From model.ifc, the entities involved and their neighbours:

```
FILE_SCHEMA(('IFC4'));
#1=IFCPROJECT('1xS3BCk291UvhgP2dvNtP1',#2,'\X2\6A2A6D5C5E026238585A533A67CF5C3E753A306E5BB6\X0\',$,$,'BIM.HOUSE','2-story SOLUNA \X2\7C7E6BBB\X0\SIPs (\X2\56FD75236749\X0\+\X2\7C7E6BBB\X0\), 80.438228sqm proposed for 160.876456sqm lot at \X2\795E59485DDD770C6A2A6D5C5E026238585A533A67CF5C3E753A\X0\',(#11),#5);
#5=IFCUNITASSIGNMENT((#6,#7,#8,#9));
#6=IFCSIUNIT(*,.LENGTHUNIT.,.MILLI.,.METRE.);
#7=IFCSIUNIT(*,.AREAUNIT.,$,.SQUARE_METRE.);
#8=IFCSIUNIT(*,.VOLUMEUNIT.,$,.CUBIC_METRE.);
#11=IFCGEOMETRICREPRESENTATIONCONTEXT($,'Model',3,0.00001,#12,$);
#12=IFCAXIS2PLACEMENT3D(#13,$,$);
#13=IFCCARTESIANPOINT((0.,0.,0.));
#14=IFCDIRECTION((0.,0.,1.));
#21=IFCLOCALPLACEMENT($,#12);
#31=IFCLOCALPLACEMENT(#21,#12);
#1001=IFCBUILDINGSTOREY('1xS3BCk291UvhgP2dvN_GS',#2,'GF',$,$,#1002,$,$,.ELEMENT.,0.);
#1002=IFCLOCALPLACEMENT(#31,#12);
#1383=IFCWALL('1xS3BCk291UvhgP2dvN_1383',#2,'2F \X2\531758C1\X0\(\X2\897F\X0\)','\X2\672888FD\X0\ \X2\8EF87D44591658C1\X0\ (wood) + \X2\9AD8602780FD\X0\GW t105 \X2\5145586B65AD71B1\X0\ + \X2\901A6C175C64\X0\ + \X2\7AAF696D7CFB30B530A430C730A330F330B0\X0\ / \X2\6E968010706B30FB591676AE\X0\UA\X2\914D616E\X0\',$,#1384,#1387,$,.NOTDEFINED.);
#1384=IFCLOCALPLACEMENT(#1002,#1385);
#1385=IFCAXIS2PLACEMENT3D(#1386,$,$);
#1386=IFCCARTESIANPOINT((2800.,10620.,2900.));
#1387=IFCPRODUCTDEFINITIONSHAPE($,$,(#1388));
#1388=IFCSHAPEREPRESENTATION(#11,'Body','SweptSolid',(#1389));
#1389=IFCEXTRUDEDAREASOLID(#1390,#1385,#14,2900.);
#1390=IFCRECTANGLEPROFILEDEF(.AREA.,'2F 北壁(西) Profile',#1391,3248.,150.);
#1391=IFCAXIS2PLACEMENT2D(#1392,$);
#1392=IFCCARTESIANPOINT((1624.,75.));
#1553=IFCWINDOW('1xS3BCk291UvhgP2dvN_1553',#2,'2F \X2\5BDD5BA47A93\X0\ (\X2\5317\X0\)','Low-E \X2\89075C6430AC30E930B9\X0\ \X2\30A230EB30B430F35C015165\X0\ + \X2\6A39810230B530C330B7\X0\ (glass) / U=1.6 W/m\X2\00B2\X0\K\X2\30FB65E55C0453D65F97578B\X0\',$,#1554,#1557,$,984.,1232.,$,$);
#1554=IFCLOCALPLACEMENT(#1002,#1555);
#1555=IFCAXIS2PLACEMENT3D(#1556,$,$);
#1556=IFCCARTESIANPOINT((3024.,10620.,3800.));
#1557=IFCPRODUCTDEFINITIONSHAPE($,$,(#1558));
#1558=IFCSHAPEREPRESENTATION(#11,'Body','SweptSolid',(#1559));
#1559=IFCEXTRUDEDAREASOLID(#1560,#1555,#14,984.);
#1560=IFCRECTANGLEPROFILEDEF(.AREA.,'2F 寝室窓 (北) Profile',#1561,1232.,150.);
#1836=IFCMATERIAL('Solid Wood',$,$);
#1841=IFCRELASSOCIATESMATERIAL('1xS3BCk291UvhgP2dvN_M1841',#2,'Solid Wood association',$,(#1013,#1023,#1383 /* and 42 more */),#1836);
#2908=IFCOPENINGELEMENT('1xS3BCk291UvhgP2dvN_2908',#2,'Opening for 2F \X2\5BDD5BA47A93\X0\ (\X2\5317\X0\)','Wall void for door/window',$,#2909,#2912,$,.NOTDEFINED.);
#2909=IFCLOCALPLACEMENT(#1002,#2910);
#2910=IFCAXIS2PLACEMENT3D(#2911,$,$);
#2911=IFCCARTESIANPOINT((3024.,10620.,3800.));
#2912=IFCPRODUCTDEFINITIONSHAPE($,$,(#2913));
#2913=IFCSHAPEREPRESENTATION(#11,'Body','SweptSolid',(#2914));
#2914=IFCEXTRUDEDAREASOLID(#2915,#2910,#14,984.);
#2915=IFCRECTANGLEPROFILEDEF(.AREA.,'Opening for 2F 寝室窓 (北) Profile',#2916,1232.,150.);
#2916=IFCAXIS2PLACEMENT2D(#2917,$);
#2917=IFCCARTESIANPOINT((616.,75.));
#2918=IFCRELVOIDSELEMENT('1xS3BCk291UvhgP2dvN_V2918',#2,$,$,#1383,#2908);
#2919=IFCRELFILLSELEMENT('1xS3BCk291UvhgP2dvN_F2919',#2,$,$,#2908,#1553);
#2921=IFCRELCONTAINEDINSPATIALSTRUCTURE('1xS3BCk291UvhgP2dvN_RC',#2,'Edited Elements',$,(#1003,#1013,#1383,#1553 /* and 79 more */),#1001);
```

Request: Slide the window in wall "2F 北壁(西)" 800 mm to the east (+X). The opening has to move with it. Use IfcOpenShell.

```python
import ifcopenshell
import ifcopenshell.api.geometry
import ifcopenshell.util.placement

model = ifcopenshell.open("model.ifc")

window = model.by_guid("1xS3BCk291UvhgP2dvN_1553")
opening = window.FillsVoids[0].RelatingOpeningElement
wall = opening.VoidsElements[0].RelatingBuildingElement

wall_matrix = ifcopenshell.util.placement.get_local_placement(wall.ObjectPlacement)
shift = wall_matrix[:3, 0] * 800.0
before = ifcopenshell.util.placement.get_local_placement(window.ObjectPlacement)[:3, 3].copy()

# The window is not placed relative to its opening, so move both.
for product in (opening, window):
    matrix = ifcopenshell.util.placement.get_local_placement(product.ObjectPlacement)
    matrix[:3, 3] += shift
    ifcopenshell.api.geometry.edit_object_placement(model, product=product, matrix=matrix, is_si=False)

after = ifcopenshell.util.placement.get_local_placement(window.ObjectPlacement)[:3, 3]
print("window moved by", (after - before).round(3) + 0.0)

model.write("model_v2.ifc")
```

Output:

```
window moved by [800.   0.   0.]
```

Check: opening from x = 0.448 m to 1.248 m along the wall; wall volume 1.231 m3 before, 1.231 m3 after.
